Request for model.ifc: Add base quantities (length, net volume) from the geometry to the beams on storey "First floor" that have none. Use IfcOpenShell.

First a look at what the model holds.

```python
import ifcopenshell
import ifcopenshell.util.element
import ifcopenshell.util.unit

model = ifcopenshell.open("model.ifc")
print(model.schema)
for unit_type in ("LENGTHUNIT", "AREAUNIT", "VOLUMEUNIT"):
    print(unit_type, ifcopenshell.util.unit.calculate_unit_scale(model, unit_type))
storey = next(s for s in model.by_type("IfcBuildingStorey") if s.Name == "First floor")
beams = [e for e in ifcopenshell.util.element.get_decomposition(storey) if e.is_a("IfcBeam")]
for e in sorted(beams, key=lambda e: e.id()):
    print(e.id(), e.is_a(), e.Name, list(ifcopenshell.util.element.get_psets(e, qtos_only=True)), sep=" | ")
```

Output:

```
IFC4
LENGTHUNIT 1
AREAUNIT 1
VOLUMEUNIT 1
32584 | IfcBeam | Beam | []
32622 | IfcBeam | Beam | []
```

```python
import ifcopenshell
import ifcopenshell.api.pset
import ifcopenshell.geom
import ifcopenshell.util.element
import ifcopenshell.util.shape
import ifcopenshell.util.unit

model = ifcopenshell.open("model.ifc")
unit_scale = ifcopenshell.util.unit.calculate_unit_scale(model)
volume_scale = ifcopenshell.util.unit.calculate_unit_scale(model, "VOLUMEUNIT")
settings = ifcopenshell.geom.settings()

storey = next(s for s in model.by_type("IfcBuildingStorey") if s.Name == "First floor")
beams = [e for e in ifcopenshell.util.element.get_decomposition(storey) if e.is_a("IfcBeam")]

for e in sorted(beams, key=lambda e: e.id()):
    if ifcopenshell.util.element.get_psets(e, qtos_only=True, should_inherit=False):
        continue
    # Geometry comes back in metres, in the element's own axes.
    shape = ifcopenshell.geom.create_shape(settings, e)
    values = {
        "Length": ifcopenshell.util.shape.get_max_xyz(shape.geometry) / unit_scale,
        "NetVolume": ifcopenshell.util.shape.get_volume(shape.geometry) / volume_scale,
    }
    qto = ifcopenshell.api.pset.add_qto(model, product=e, name="Qto_BeamBaseQuantities")
    ifcopenshell.api.pset.edit_qto(model, qto=qto, properties=values)
    print(e.id(), {k: round(v, 3) for k, v in values.items()})

model.write("model-out.ifc")
```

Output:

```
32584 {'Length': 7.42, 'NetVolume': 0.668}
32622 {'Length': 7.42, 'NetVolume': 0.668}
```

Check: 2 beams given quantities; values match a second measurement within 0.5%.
